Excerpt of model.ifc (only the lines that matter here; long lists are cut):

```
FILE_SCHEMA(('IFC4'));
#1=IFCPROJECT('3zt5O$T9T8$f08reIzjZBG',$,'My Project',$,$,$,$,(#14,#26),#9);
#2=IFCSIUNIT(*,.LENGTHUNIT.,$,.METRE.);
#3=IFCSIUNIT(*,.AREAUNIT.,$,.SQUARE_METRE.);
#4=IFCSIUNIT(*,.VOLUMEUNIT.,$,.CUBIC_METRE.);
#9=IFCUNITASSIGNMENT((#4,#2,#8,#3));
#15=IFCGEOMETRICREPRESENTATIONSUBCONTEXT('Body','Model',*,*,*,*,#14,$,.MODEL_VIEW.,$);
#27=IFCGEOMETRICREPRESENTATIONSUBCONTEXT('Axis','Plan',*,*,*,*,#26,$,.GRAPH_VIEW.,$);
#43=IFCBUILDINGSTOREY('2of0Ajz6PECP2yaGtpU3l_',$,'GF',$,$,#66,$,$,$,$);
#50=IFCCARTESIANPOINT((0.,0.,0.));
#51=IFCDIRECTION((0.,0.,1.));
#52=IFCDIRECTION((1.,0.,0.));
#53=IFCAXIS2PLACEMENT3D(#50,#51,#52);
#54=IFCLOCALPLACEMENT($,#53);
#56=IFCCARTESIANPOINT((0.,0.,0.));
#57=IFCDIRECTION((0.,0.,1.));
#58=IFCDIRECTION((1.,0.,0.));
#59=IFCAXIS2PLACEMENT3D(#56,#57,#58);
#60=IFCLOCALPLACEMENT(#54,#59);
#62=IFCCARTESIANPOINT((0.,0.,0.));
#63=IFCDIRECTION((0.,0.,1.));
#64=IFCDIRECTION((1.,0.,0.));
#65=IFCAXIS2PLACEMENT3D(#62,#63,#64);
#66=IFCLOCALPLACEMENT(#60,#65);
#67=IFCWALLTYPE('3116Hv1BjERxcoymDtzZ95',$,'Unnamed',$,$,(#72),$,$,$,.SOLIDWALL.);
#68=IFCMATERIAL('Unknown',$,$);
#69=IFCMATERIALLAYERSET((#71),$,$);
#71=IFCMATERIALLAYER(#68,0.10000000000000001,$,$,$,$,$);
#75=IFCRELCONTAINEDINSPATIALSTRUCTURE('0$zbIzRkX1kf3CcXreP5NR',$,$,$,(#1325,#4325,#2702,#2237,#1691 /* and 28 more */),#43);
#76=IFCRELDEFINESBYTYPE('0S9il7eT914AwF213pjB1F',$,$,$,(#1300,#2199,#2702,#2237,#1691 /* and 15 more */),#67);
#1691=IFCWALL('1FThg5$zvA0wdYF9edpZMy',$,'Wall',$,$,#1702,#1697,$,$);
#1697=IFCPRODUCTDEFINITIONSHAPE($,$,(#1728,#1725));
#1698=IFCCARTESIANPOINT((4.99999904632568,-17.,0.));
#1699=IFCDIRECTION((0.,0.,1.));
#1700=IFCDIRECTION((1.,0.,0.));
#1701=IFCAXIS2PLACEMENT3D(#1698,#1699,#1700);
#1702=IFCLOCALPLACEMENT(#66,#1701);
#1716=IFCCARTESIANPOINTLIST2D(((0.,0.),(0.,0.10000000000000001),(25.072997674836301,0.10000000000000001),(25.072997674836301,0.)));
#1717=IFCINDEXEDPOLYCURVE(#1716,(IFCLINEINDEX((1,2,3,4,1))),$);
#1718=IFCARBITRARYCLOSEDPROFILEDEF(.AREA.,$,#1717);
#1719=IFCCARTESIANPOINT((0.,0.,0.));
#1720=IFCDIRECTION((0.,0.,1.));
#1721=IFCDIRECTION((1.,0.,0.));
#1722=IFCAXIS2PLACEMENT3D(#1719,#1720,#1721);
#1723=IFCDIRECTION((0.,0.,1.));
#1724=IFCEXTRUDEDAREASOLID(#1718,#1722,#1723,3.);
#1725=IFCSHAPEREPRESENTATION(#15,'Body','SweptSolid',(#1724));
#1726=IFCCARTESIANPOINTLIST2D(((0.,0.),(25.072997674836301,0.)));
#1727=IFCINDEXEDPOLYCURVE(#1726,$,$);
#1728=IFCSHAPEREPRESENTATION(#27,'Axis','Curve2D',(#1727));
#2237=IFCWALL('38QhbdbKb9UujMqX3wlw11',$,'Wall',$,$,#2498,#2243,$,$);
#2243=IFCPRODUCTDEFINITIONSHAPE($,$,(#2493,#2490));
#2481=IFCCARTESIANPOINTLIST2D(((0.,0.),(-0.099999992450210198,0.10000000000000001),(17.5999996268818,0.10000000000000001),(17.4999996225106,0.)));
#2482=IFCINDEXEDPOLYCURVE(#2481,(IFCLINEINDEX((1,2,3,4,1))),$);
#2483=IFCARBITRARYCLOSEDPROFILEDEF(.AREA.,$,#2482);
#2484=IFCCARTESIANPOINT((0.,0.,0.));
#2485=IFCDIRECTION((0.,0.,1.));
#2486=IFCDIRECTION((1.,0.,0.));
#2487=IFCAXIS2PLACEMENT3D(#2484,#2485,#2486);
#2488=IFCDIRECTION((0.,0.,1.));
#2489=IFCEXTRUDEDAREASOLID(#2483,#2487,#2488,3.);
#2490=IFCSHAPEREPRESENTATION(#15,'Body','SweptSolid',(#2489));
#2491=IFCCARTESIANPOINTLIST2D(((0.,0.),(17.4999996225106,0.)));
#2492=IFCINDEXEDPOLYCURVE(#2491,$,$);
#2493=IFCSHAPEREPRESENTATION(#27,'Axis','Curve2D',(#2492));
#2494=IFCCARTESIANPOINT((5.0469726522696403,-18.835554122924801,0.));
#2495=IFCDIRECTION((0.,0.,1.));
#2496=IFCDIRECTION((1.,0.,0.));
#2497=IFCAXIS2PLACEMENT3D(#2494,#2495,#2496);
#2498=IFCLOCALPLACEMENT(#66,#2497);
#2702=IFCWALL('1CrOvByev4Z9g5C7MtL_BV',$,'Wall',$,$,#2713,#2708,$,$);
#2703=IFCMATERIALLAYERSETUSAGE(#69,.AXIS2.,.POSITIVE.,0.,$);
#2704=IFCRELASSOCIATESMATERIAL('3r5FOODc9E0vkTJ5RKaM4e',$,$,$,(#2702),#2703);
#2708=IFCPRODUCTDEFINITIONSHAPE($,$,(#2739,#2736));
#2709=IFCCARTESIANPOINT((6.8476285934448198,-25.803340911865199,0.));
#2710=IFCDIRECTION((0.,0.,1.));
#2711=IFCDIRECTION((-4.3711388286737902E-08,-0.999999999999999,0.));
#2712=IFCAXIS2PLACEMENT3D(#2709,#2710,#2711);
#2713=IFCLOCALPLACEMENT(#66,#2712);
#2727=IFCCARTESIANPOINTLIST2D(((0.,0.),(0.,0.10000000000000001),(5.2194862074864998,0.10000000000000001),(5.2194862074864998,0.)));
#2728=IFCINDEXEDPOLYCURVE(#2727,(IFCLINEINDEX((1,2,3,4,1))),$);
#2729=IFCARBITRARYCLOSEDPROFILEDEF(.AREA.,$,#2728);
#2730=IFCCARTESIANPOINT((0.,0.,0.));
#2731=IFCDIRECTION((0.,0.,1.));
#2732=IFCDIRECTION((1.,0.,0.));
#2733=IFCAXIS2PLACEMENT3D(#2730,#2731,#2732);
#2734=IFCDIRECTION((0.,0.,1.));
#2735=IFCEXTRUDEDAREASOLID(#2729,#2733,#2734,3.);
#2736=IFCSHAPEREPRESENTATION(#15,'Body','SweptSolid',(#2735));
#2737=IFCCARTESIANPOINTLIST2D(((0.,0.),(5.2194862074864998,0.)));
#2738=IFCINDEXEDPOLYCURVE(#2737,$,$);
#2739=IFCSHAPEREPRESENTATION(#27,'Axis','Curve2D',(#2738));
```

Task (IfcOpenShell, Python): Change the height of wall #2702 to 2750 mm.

```python
import ifcopenshell
import ifcopenshell.geom
import ifcopenshell.util.representation
import ifcopenshell.util.shape

model = ifcopenshell.open("model.ifc")
settings = ifcopenshell.geom.settings()


def volume(element):
    """Net volume in cubic metres, openings subtracted."""
    shape = ifcopenshell.geom.create_shape(settings, element)
    return ifcopenshell.util.shape.get_volume(shape.geometry)


wall = model.by_id(2702)
before = volume(wall)

body = ifcopenshell.util.representation.get_representation(wall, "Model", "Body")
solid = body.Items[0]
old_height = solid.Depth
solid.Depth = 2.75
after = volume(wall)

print(f"height {old_height:g} -> {solid.Depth:g}, volume {before:.3f} -> {after:.3f} m3")

model.write("model-out.ifc")
```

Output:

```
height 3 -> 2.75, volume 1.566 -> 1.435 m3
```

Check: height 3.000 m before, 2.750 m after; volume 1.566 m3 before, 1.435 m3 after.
